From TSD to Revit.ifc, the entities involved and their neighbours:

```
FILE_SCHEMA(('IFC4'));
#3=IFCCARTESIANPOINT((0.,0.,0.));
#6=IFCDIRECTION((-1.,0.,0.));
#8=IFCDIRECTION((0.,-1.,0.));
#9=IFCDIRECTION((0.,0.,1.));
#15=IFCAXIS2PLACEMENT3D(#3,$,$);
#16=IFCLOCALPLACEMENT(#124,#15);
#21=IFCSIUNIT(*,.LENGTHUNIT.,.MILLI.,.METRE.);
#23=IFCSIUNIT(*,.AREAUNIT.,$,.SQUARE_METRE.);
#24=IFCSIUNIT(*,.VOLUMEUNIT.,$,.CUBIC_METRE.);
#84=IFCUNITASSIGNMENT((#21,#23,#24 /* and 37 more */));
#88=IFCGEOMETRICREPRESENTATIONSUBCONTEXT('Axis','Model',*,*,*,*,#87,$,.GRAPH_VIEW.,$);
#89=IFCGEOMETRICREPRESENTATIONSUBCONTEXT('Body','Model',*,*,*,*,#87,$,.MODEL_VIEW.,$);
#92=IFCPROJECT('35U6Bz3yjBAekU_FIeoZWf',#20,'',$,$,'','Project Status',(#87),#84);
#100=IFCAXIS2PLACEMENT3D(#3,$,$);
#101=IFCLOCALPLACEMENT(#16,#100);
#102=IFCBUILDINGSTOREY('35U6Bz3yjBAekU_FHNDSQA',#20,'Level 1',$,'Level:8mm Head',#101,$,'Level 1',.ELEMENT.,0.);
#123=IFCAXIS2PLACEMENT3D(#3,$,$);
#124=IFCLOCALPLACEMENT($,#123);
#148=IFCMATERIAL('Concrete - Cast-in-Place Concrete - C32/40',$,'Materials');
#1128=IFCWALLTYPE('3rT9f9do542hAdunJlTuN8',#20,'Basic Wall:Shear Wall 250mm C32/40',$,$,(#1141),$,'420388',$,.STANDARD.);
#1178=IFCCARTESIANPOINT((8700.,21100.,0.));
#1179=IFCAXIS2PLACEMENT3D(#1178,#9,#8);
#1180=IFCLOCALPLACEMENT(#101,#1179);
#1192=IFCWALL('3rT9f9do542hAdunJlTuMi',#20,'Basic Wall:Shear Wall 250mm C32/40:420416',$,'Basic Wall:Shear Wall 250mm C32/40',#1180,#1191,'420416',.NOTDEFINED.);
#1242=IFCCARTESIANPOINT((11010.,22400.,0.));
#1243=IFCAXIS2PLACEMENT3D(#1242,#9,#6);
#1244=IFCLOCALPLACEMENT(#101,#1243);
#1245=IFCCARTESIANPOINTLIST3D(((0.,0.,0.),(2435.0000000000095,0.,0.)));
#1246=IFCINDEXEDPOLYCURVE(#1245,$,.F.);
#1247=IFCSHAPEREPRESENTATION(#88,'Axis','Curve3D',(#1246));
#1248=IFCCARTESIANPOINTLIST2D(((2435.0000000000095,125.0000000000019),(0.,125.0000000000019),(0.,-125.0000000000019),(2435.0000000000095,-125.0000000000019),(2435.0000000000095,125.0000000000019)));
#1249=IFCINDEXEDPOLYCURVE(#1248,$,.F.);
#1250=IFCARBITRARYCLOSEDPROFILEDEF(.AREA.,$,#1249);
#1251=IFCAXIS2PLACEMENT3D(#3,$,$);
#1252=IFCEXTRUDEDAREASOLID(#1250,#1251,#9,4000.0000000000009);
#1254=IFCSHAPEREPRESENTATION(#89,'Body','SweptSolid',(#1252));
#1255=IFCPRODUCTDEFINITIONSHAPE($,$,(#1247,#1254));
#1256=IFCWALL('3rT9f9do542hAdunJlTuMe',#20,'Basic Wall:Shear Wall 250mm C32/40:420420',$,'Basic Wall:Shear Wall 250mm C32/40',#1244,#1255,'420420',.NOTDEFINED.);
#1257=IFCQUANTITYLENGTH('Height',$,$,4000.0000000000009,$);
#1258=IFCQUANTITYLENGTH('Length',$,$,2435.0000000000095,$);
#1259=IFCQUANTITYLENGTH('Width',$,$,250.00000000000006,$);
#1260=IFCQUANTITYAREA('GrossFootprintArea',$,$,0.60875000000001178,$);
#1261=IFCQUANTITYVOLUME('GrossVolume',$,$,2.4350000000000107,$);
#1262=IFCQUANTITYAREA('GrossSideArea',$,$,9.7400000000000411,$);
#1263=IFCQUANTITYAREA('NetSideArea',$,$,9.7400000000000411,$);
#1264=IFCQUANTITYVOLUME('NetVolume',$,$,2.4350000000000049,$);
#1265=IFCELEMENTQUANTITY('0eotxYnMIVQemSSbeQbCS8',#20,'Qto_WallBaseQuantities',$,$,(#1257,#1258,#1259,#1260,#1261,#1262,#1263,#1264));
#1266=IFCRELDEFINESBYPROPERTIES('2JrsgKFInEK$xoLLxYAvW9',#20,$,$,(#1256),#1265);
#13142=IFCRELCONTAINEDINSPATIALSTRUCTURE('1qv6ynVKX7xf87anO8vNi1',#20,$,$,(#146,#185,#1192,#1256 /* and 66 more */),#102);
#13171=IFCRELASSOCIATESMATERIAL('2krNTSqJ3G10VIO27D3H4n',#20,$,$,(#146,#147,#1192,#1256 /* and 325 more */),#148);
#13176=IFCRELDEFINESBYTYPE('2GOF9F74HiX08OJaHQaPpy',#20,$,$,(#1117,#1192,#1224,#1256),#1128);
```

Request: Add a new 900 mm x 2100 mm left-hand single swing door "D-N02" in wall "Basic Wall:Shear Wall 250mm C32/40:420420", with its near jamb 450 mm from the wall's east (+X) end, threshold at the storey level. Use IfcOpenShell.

```python
import numpy as np
import ifcopenshell
import ifcopenshell.api.feature
import ifcopenshell.api.geometry
import ifcopenshell.api.pset
import ifcopenshell.api.root
import ifcopenshell.api.spatial
import ifcopenshell.geom
import ifcopenshell.util.element
import ifcopenshell.util.placement
import ifcopenshell.util.representation
import ifcopenshell.util.shape
import ifcopenshell.util.unit

model = ifcopenshell.open("TSD to Revit.ifc")
unit_scale = ifcopenshell.util.unit.calculate_unit_scale(model)
area_scale = ifcopenshell.util.unit.calculate_unit_scale(model, "AREAUNIT")
volume_scale = ifcopenshell.util.unit.calculate_unit_scale(model, "VOLUMEUNIT")
settings = ifcopenshell.geom.settings()


def volume(element):
    """Net volume in cubic metres, openings subtracted."""
    shape = ifcopenshell.geom.create_shape(settings, element)
    return ifcopenshell.util.shape.get_volume(shape.geometry)


wall = model.by_guid("3rT9f9do542hAdunJlTuMe")
storey = ifcopenshell.util.element.get_container(wall, ifc_class="IfcBuildingStorey")
context = ifcopenshell.util.representation.get_context(model, "Model", "Body", "MODEL_VIEW")
before = volume(wall)

width, height, from_end, sill = 0.9, 2.1, 0.45, 0.0  # metres

# The wall runs along its own X axis, and the end named is its -X end.
wall_shape = ifcopenshell.geom.create_shape(settings, wall)
x, y, z = ifcopenshell.util.shape.get_vertices(wall_shape.geometry).T
start = x.min() + from_end
face, thickness = float(y.min()), float(y.max() - y.min())
wall_matrix = ifcopenshell.util.placement.get_local_placement(wall.ObjectPlacement)
level = ifcopenshell.util.placement.get_local_placement(storey.ObjectPlacement)[2, 3]


def in_wall(x, y):
    """Placement at x, y metres in the wall's axes, at sill height."""
    matrix = wall_matrix.copy()
    matrix[:, 3] = wall_matrix @ np.array([x / unit_scale, y / unit_scale, 0.0, 1.0])
    matrix[2, 3] = level + sill / unit_scale
    return matrix


# Opening: a box that overshoots both wall faces by 50 mm.
opening = ifcopenshell.api.root.create_entity(model, ifc_class="IfcOpeningElement", predefined_type="OPENING")
box = ifcopenshell.api.geometry.add_wall_representation(
    model, context=context, length=width, height=height, thickness=thickness + 0.1
)
ifcopenshell.api.geometry.assign_representation(model, product=opening, representation=box)
ifcopenshell.api.geometry.edit_object_placement(model, product=opening, matrix=in_wall(start, face - 0.05), is_si=False)
ifcopenshell.api.feature.add_feature(model, feature=opening, element=wall)

door = ifcopenshell.api.root.create_entity(model, ifc_class="IfcDoor", name="D-N02", predefined_type="DOOR")
door.OverallWidth, door.OverallHeight = width / unit_scale, height / unit_scale
door.OperationType = "SINGLE_SWING_LEFT"
body = ifcopenshell.api.geometry.add_door_representation(
    model,
    context=context,
    overall_width=door.OverallWidth,
    overall_height=door.OverallHeight,
    operation_type="SINGLE_SWING_LEFT",
    lining_properties={"LiningDepth": thickness / unit_scale, "ThresholdDepth": thickness / unit_scale},
)
ifcopenshell.api.geometry.assign_representation(model, product=door, representation=body)
ifcopenshell.api.spatial.assign_container(model, products=[door], relating_structure=storey)
ifcopenshell.api.feature.add_filling(model, opening=opening, element=door)

# The lining spans the wall, so the door starts at the wall face.
ifcopenshell.api.geometry.edit_object_placement(model, product=door, matrix=in_wall(start, face), is_si=False)

after = volume(wall)

# Update the wall's stored quantities.
qto = model.by_id(ifcopenshell.util.element.get_pset(wall, "Qto_WallBaseQuantities", should_inherit=False)["id"])
ifcopenshell.api.pset.edit_qto(model, qto=qto, properties={
    "NetSideArea": after / thickness / area_scale,
    "NetVolume": after / volume_scale,
})

print(f"wall volume {before:.3f} -> {after:.3f} m3")

model.write("TSD to Revit_v2.ifc")
```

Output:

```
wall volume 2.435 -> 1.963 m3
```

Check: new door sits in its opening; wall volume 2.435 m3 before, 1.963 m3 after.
